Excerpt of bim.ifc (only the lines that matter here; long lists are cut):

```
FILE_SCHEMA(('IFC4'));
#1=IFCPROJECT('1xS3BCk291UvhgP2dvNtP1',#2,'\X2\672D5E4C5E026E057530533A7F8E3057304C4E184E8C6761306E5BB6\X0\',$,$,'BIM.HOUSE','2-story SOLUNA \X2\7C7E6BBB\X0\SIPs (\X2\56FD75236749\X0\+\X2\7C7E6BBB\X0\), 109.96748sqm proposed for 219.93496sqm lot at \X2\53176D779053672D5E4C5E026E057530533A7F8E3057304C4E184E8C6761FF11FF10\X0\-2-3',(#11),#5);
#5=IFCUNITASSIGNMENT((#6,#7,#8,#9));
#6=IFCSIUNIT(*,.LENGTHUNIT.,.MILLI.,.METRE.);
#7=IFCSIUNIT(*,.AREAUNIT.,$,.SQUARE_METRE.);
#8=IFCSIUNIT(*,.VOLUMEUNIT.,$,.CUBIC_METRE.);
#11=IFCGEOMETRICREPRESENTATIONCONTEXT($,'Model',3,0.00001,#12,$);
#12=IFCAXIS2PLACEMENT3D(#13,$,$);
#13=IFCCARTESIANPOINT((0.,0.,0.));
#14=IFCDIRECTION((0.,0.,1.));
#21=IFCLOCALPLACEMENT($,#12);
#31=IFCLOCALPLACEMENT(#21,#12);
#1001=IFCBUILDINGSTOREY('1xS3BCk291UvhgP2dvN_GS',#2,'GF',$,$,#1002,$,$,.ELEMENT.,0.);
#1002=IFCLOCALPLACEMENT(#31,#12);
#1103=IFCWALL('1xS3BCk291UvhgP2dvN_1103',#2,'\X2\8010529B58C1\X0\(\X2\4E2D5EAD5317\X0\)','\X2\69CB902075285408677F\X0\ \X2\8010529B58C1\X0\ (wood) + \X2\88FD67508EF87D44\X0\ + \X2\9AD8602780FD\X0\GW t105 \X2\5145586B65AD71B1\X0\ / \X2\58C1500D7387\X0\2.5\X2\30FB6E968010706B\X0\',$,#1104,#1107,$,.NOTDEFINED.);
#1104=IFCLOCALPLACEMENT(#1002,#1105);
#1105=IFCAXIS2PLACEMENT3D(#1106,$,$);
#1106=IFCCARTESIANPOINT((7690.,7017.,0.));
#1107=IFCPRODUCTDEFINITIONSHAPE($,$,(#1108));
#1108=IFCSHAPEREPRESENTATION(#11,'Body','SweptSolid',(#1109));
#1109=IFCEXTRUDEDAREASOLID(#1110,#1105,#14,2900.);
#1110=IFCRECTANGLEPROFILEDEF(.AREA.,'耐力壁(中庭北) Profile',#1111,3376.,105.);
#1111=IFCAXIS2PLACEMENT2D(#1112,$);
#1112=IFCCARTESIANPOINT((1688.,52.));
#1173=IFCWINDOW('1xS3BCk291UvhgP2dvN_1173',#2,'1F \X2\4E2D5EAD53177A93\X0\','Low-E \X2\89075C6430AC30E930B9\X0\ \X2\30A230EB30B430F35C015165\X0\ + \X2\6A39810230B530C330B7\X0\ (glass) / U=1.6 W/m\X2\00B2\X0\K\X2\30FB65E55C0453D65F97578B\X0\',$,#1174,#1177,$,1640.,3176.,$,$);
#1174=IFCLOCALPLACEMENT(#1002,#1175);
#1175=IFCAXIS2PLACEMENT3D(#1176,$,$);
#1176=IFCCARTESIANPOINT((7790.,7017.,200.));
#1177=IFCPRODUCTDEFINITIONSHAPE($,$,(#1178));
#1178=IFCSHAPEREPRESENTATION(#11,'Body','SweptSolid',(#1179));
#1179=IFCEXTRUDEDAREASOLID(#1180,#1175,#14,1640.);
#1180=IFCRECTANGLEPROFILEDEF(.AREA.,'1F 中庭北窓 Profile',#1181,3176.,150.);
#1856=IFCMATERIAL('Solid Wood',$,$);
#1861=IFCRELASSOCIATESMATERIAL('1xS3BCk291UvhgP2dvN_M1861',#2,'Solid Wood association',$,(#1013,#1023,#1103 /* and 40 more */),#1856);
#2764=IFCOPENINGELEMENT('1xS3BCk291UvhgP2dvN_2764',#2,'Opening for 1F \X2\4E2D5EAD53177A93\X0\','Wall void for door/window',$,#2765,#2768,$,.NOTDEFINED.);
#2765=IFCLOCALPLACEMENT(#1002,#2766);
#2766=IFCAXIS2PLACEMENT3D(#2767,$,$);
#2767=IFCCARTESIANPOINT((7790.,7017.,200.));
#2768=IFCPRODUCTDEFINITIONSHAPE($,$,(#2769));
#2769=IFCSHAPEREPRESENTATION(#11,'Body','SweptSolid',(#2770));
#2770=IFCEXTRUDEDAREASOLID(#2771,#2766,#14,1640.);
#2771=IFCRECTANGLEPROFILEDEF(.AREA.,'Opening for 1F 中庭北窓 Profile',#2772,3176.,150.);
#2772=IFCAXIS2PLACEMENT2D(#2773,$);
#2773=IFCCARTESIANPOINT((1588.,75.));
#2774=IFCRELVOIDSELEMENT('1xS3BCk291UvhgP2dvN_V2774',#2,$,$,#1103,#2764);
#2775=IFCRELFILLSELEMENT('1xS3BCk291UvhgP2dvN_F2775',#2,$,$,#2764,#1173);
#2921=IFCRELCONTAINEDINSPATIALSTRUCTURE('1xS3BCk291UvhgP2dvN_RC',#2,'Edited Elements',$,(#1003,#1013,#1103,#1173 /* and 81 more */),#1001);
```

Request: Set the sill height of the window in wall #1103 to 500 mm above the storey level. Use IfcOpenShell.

```python
import numpy as np
import ifcopenshell
import ifcopenshell.api.geometry
import ifcopenshell.geom
import ifcopenshell.util.element
import ifcopenshell.util.placement
import ifcopenshell.util.shape
import ifcopenshell.util.unit

model = ifcopenshell.open("bim.ifc")
unit_scale = ifcopenshell.util.unit.calculate_unit_scale(model)

window = model.by_guid("1xS3BCk291UvhgP2dvN_1173")
opening = window.FillsVoids[0].RelatingOpeningElement
storey = ifcopenshell.util.element.get_container(window, ifc_class="IfcBuildingStorey")
level = ifcopenshell.util.placement.get_local_placement(storey.ObjectPlacement)[2, 3]

# The opening's origin need not be at the sill, so measure its lowest point.
shape = ifcopenshell.geom.create_shape(ifcopenshell.geom.settings(), opening)
bottom = ifcopenshell.util.shape.get_shape_bottom_elevation(shape, shape.geometry) / unit_scale
dz = level + 500.0 - bottom

shift = np.array([0.0, 0.0, dz])
# The window is not placed relative to its opening, so move both.
for product in (opening, window):
    matrix = ifcopenshell.util.placement.get_local_placement(product.ObjectPlacement)
    matrix[:3, 3] += shift
    ifcopenshell.api.geometry.edit_object_placement(model, product=product, matrix=matrix, is_si=False)

print(f"moved by {dz * unit_scale:+.3f} m")

model.write("bim_edited.ifc")
```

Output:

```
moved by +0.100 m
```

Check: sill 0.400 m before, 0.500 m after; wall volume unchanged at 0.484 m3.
